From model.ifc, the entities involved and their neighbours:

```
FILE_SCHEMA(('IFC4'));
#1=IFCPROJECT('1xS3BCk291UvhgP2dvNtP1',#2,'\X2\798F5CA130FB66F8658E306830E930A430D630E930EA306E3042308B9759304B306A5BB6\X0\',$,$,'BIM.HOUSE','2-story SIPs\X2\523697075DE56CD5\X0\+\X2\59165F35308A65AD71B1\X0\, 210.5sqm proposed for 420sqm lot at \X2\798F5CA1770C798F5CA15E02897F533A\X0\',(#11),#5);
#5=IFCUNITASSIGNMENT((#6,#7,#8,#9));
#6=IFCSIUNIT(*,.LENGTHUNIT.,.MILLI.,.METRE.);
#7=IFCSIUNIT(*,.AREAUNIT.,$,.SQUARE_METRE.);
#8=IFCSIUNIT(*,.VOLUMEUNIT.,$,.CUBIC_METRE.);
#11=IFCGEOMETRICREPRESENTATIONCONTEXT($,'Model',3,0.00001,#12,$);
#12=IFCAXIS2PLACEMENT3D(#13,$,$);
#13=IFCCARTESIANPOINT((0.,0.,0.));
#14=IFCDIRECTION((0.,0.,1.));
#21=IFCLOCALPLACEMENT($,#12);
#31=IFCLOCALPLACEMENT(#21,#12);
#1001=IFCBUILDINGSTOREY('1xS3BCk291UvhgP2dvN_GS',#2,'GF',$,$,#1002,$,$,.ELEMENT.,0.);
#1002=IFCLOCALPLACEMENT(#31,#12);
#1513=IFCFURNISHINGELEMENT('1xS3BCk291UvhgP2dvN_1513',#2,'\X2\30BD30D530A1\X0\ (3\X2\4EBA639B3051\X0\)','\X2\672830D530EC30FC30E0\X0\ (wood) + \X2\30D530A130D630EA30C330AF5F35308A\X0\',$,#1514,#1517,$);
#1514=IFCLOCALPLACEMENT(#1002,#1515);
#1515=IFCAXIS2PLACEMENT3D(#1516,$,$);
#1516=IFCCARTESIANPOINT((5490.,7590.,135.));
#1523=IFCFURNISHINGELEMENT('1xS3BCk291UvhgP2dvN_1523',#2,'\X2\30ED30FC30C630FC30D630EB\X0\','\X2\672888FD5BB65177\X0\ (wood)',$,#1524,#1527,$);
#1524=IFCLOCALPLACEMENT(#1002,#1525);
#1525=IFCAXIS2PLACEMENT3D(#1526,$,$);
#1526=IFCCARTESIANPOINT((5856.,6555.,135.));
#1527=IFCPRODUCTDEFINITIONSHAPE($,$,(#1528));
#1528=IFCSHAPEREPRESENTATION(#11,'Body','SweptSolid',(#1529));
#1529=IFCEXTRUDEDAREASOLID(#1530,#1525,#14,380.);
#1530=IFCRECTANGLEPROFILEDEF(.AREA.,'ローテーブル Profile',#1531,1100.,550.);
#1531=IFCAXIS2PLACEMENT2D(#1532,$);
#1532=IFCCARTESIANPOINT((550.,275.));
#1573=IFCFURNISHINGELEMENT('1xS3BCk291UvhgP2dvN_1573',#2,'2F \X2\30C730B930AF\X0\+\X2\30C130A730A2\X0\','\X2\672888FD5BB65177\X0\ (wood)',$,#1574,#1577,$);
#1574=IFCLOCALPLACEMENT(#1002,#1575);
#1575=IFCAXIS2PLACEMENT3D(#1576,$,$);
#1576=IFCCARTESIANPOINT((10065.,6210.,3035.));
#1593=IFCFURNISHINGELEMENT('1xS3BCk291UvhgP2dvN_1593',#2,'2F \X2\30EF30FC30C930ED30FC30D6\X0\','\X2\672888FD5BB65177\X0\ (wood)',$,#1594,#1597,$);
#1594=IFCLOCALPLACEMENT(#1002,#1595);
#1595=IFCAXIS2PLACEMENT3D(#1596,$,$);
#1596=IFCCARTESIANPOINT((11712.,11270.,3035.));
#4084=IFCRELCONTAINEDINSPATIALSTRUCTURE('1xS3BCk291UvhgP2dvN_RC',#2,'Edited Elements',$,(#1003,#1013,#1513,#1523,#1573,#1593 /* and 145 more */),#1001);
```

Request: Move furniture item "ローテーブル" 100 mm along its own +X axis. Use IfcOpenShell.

```python
import ifcopenshell
import ifcopenshell.api.geometry
import ifcopenshell.util.placement
import ifcopenshell.util.unit

model = ifcopenshell.open("model.ifc")
unit_scale = ifcopenshell.util.unit.calculate_unit_scale(model)

item = model.by_guid("1xS3BCk291UvhgP2dvN_1523")
matrix = ifcopenshell.util.placement.get_local_placement(item.ObjectPlacement)
matrix[:3, 3] += matrix[:3, 0] * 0.1 / unit_scale
ifcopenshell.api.geometry.edit_object_placement(model, product=item, matrix=matrix, is_si=False)

print(ifcopenshell.util.placement.get_local_placement(item.ObjectPlacement).round(3) + 0.0)

model.write("model_edited.ifc")
```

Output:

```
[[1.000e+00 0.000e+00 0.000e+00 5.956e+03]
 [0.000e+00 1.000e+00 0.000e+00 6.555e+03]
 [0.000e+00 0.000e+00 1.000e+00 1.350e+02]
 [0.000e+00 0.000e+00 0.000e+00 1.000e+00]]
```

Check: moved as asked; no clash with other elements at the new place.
